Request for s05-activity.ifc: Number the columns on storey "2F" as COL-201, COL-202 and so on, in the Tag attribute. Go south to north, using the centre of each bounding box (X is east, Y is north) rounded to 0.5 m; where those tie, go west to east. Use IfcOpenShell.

First a look at what the model holds.

```python
import ifcopenshell
import ifcopenshell.util.element
import ifcopenshell.util.placement

model = ifcopenshell.open("s05-activity.ifc")
print(model.schema)
storey = next(s for s in model.by_type("IfcBuildingStorey") if s.Name == "2F")
columns = [e for e in ifcopenshell.util.element.get_decomposition(storey) if e.is_a("IfcColumn")]
for e in sorted(columns, key=lambda e: e.id()):
    origin = ifcopenshell.util.placement.get_local_placement(e.ObjectPlacement)[:3, 3]
    print(e.id(), e.Tag, e.Name, origin.round(2) + 0.0, sep=" | ")
```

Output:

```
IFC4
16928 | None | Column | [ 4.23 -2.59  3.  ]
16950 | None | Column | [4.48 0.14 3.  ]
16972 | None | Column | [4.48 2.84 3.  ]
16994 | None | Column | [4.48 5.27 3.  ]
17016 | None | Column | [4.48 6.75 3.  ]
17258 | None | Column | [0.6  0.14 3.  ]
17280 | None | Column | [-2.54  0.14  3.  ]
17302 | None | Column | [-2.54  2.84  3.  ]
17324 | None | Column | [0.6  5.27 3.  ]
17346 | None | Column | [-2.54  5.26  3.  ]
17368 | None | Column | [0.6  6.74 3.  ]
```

```python
import ifcopenshell
import ifcopenshell.geom
import ifcopenshell.util.element
import ifcopenshell.util.shape

model = ifcopenshell.open("s05-activity.ifc")
settings = ifcopenshell.geom.settings()
settings.set("use-world-coords", True)


def centre(element):
    shape = ifcopenshell.geom.create_shape(settings, element)
    return ifcopenshell.util.shape.get_bbox_centroid(shape.geometry)


storey = next(s for s in model.by_type("IfcBuildingStorey") if s.Name == "2F")
columns = [e for e in ifcopenshell.util.element.get_decomposition(storey) if e.is_a("IfcColumn")]

# Insertion points can sit at a corner or the storey origin, so sort by the geometry (in metres).
centres = {e: centre(e) for e in columns}
columns.sort(key=lambda e: (round(centres[e][1] / 0.5), centres[e][0]))

for i, e in enumerate(columns, start=1):
    number = f"COL-2{i:02d}"
    e.Tag = number
    print(e.id(), number)

model.write("s05-activity_edited.ifc")
```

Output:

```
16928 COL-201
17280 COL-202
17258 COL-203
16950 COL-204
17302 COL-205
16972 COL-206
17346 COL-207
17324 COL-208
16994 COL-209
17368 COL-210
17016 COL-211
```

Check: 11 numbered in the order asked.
